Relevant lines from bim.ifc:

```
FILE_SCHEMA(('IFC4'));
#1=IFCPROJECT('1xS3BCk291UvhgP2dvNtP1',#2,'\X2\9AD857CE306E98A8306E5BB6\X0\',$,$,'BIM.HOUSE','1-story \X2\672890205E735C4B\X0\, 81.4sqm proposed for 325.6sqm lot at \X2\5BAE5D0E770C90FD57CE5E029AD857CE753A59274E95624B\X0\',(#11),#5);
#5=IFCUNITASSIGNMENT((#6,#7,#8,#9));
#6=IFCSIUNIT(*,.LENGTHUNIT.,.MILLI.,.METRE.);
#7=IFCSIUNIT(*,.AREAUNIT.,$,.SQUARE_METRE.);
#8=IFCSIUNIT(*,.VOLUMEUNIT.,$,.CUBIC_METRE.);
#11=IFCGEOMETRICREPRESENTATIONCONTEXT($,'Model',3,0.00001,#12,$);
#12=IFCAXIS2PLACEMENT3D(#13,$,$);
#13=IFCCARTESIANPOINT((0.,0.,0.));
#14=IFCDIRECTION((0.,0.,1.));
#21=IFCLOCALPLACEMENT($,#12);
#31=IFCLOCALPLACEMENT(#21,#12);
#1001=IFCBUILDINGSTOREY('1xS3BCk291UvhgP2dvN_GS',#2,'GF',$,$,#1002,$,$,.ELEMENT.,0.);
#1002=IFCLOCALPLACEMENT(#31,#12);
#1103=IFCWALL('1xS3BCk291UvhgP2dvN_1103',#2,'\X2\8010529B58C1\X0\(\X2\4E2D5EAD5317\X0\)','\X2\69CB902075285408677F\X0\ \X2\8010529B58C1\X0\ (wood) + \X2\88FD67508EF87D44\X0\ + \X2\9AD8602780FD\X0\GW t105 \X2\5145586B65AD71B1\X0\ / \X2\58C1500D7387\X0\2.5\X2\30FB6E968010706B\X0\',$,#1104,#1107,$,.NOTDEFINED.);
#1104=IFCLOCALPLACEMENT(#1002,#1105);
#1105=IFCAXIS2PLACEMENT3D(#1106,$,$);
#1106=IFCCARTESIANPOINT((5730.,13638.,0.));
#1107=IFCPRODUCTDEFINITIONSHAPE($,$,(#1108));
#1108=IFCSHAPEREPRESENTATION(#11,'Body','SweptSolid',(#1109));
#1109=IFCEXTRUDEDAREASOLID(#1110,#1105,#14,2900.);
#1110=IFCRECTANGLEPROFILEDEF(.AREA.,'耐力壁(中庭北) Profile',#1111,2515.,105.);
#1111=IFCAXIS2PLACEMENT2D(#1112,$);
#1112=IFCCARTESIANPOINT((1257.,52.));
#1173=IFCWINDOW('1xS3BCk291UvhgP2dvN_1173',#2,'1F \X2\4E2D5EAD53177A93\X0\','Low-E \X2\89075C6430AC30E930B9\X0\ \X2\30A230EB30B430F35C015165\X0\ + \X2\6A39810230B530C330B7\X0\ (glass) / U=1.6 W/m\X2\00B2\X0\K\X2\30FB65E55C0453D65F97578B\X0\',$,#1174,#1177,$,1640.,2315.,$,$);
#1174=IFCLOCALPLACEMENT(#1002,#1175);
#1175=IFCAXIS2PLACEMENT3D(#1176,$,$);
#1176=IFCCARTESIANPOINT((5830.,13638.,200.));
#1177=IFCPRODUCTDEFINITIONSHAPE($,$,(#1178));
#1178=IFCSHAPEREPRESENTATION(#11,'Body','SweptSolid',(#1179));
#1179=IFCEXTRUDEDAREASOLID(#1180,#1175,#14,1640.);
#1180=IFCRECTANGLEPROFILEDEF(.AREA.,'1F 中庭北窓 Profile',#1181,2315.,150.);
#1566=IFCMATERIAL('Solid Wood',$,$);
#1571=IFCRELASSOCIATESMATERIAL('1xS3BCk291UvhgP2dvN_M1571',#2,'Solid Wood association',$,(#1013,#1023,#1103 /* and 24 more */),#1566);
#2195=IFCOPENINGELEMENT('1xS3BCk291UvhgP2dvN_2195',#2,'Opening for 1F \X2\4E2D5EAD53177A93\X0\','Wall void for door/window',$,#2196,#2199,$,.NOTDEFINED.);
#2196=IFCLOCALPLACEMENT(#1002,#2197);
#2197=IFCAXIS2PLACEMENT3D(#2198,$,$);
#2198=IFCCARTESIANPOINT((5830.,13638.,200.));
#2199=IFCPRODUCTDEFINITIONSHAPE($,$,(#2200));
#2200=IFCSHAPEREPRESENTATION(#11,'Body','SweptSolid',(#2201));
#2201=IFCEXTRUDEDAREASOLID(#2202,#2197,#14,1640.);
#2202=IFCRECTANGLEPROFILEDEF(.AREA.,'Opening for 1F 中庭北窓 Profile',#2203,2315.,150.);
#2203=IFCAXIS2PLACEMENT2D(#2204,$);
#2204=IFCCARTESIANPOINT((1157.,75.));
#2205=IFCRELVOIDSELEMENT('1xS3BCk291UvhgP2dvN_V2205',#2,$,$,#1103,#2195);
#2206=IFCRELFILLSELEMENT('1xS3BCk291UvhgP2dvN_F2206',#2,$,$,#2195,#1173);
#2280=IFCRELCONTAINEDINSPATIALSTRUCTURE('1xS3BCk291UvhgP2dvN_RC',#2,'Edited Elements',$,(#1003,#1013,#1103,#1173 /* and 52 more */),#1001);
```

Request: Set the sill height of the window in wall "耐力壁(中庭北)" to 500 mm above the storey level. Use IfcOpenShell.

```python
import numpy as np
import ifcopenshell
import ifcopenshell.api.geometry
import ifcopenshell.geom
import ifcopenshell.util.element
import ifcopenshell.util.placement
import ifcopenshell.util.shape
import ifcopenshell.util.unit

model = ifcopenshell.open("bim.ifc")
unit_scale = ifcopenshell.util.unit.calculate_unit_scale(model)

window = model.by_guid("1xS3BCk291UvhgP2dvN_1173")
opening = window.FillsVoids[0].RelatingOpeningElement
storey = ifcopenshell.util.element.get_container(window, ifc_class="IfcBuildingStorey")
level = ifcopenshell.util.placement.get_local_placement(storey.ObjectPlacement)[2, 3]

# The opening's origin need not be at the sill, so measure its lowest point.
shape = ifcopenshell.geom.create_shape(ifcopenshell.geom.settings(), opening)
bottom = ifcopenshell.util.shape.get_shape_bottom_elevation(shape, shape.geometry) / unit_scale
dz = level + 0.5 / unit_scale - bottom

shift = np.array([0.0, 0.0, dz])
# The window is not placed relative to its opening, so move both.
for product in (opening, window):
    matrix = ifcopenshell.util.placement.get_local_placement(product.ObjectPlacement)
    matrix[:3, 3] += shift
    ifcopenshell.api.geometry.edit_object_placement(model, product=product, matrix=matrix, is_si=False)

print(f"moved by {dz * unit_scale:+.3f} m")

model.write("bim_updated.ifc")
```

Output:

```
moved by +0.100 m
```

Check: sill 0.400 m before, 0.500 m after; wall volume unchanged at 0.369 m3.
